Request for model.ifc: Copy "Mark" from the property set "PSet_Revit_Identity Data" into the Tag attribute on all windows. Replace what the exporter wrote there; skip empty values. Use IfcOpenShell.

First a look at what the model holds.

```python
import ifcopenshell
import ifcopenshell.util.element

model = ifcopenshell.open("model.ifc")
print(model.schema)
windows = model.by_type("IfcWindow")
print(len(windows), "windows")
for e in windows[:8]:
    source = ifcopenshell.util.element.get_pset(e, "PSet_Revit_Identity Data", "Mark")
    target = e.Tag
    print(e.id(), repr(source), repr(target), sep=" | ")
```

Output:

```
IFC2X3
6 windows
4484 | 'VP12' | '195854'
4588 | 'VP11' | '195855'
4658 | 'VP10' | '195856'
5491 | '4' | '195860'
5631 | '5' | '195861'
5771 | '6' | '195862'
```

```python
import ifcopenshell
import ifcopenshell.util.element

model = ifcopenshell.open("model.ifc")

count = 0
for e in model.by_type("IfcWindow"):
    value = ifcopenshell.util.element.get_pset(e, "PSet_Revit_Identity Data", "Mark")
    current = e.Tag
    if not value or not value.strip() or current == value:
        continue
    e.Tag = value
    count += 1

print(count, "windows updated")

model.write("model_rev.ifc")
```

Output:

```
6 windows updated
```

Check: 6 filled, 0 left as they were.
